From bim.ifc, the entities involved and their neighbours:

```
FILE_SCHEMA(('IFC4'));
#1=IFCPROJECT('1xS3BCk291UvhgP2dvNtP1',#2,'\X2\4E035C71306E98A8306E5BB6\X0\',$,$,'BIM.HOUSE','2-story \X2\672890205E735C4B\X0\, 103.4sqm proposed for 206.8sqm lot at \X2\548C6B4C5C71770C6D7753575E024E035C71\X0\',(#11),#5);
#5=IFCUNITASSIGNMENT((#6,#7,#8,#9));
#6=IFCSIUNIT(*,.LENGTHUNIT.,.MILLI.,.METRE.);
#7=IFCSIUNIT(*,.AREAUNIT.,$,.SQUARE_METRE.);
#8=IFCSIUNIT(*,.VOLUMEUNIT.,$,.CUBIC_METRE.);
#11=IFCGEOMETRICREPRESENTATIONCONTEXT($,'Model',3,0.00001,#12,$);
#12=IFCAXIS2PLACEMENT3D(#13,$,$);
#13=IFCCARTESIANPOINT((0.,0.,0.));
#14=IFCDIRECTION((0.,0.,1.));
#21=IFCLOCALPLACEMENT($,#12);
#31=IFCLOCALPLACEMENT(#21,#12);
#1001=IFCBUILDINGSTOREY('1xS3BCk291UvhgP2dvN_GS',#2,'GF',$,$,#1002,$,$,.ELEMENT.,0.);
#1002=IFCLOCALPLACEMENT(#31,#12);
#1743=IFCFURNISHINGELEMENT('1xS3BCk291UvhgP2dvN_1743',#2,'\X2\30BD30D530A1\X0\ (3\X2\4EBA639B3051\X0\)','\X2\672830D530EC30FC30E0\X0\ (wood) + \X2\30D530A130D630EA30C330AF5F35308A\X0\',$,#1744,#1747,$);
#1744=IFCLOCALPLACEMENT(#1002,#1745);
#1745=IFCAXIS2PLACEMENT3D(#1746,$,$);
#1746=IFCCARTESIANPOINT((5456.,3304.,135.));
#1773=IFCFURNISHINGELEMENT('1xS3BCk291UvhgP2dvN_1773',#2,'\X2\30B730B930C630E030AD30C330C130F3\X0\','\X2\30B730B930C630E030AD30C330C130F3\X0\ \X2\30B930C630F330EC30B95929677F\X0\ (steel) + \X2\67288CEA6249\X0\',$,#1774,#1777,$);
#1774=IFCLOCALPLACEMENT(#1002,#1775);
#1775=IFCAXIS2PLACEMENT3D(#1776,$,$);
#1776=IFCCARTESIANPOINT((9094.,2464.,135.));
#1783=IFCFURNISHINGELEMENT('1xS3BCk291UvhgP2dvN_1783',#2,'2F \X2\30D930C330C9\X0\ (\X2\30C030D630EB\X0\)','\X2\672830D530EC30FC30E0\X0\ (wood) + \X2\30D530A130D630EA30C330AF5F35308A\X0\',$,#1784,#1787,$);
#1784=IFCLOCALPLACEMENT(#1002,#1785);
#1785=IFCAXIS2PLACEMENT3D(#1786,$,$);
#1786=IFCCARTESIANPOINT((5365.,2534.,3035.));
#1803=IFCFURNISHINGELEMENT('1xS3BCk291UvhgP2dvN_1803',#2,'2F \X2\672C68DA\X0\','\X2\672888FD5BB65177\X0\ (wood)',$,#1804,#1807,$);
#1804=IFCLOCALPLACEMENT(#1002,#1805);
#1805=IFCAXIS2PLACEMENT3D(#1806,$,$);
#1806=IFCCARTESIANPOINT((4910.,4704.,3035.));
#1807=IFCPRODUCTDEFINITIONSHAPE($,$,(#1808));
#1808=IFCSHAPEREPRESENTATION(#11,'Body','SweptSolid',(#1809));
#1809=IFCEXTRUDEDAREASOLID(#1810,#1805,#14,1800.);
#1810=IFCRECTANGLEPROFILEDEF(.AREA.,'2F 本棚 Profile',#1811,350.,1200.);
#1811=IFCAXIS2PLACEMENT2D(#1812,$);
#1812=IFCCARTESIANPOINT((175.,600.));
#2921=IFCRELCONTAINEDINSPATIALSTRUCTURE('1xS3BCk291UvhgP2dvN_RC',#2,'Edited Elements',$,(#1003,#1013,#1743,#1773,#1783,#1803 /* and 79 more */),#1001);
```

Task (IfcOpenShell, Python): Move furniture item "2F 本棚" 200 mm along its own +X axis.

```python
import ifcopenshell
import ifcopenshell.api.geometry
import ifcopenshell.util.placement

model = ifcopenshell.open("bim.ifc")

item = model.by_id(1803)
matrix = ifcopenshell.util.placement.get_local_placement(item.ObjectPlacement)
matrix[:3, 3] += matrix[:3, 0] * 200.0
ifcopenshell.api.geometry.edit_object_placement(model, product=item, matrix=matrix, is_si=False)

print(ifcopenshell.util.placement.get_local_placement(item.ObjectPlacement).round(3) + 0.0)

model.write("bim_rev.ifc")
```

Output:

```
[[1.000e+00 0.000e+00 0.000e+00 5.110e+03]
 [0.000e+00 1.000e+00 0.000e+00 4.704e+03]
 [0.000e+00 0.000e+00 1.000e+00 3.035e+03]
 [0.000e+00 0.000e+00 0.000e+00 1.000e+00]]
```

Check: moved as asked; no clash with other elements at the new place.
